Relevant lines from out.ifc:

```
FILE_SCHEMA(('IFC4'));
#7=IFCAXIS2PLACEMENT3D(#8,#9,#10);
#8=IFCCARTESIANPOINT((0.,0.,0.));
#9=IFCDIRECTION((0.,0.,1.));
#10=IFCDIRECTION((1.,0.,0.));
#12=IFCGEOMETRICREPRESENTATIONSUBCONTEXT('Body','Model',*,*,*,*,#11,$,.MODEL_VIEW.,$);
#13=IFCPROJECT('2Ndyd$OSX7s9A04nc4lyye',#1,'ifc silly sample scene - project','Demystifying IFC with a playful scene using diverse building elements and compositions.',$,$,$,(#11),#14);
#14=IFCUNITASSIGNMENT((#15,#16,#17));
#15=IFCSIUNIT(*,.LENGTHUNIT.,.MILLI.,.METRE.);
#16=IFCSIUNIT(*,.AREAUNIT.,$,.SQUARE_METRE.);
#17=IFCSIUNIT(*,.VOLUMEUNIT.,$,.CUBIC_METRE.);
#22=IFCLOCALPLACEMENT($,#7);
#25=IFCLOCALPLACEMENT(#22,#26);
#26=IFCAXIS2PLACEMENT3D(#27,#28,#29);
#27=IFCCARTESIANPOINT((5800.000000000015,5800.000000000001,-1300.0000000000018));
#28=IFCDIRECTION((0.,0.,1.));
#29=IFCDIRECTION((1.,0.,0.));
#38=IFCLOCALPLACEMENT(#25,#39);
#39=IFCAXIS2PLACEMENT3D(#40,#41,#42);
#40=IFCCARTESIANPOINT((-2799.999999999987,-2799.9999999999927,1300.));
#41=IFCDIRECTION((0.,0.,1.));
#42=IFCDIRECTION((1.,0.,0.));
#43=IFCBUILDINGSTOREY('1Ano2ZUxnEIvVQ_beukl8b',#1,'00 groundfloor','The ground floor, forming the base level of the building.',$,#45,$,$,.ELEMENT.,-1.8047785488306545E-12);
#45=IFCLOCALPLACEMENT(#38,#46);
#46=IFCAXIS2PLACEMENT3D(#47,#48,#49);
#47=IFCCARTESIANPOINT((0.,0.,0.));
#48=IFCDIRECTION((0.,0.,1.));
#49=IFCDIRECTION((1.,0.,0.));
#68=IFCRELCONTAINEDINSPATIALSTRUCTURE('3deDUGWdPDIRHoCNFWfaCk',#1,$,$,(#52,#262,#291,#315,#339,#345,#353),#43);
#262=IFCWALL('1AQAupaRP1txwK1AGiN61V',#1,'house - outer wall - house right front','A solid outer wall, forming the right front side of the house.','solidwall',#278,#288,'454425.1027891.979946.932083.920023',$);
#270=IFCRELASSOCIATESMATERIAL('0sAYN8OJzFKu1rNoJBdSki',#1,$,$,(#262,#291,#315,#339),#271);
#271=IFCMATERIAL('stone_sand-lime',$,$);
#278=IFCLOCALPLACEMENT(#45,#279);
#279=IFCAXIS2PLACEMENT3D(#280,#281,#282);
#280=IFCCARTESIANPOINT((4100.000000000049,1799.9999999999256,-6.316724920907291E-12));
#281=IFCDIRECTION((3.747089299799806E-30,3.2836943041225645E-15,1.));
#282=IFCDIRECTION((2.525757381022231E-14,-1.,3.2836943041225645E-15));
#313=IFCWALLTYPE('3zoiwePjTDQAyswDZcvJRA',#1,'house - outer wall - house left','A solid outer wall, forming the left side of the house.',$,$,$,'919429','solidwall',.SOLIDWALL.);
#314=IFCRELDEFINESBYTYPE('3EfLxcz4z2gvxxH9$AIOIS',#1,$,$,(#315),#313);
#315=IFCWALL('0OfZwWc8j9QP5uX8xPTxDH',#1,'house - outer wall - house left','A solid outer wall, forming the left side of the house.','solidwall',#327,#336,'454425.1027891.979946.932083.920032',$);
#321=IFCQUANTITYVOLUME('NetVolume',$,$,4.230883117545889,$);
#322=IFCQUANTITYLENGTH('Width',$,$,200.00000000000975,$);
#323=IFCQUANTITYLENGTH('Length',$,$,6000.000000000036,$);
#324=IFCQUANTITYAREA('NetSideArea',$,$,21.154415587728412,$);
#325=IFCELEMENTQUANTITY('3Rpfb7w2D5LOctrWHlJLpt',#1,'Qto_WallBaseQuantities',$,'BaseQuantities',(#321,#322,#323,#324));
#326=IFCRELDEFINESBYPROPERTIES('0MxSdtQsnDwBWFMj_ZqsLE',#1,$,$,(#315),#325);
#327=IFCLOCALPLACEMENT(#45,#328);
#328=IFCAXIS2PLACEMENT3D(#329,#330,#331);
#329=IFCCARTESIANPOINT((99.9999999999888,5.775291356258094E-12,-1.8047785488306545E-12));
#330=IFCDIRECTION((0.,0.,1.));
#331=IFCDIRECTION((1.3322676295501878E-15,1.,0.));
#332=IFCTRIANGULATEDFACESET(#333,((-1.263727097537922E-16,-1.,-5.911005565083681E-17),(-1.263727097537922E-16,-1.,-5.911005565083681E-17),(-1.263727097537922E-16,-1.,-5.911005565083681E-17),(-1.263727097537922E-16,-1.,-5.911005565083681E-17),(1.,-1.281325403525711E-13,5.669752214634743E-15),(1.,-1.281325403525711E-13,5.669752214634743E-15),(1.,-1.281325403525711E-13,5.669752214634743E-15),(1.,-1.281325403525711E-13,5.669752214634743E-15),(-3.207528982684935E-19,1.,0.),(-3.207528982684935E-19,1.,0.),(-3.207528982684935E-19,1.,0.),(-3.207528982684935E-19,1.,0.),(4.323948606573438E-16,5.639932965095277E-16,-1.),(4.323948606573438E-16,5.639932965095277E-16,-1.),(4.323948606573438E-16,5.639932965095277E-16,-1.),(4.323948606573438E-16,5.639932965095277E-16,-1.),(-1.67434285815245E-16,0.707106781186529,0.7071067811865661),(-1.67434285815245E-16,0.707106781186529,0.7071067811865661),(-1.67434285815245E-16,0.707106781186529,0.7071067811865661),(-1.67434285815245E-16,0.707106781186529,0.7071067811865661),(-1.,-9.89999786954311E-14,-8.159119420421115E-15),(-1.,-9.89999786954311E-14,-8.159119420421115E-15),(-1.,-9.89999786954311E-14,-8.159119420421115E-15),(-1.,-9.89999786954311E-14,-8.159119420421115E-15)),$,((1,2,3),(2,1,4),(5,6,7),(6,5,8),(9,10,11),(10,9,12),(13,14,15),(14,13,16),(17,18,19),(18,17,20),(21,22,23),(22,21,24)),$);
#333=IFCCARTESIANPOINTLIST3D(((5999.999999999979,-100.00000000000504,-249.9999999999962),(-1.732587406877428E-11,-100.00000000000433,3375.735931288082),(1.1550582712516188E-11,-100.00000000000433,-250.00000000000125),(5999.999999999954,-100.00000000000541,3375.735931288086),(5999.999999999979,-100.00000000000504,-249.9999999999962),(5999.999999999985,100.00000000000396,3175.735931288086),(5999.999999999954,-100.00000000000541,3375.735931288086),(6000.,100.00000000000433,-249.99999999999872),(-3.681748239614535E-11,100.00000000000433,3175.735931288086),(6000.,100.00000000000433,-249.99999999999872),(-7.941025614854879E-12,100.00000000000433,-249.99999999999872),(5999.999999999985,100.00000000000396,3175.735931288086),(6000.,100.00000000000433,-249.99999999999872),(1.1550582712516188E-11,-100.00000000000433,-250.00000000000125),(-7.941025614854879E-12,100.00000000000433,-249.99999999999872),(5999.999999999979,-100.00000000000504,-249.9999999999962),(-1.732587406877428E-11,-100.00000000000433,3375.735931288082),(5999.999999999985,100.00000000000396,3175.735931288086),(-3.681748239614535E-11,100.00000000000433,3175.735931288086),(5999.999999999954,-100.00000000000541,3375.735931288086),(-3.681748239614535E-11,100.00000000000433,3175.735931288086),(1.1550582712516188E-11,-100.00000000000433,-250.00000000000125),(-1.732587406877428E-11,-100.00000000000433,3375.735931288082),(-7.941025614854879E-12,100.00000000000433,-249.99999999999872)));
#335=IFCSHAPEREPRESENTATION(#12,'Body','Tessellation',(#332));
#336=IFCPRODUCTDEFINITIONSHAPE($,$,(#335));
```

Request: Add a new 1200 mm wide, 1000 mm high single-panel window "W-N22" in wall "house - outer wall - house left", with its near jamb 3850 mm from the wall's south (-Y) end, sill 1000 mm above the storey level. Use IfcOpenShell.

```python
import numpy as np
import ifcopenshell
import ifcopenshell.api.feature
import ifcopenshell.api.geometry
import ifcopenshell.api.pset
import ifcopenshell.api.root
import ifcopenshell.api.spatial
import ifcopenshell.geom
import ifcopenshell.util.element
import ifcopenshell.util.placement
import ifcopenshell.util.representation
import ifcopenshell.util.shape
import ifcopenshell.util.unit

model = ifcopenshell.open("out.ifc")
unit_scale = ifcopenshell.util.unit.calculate_unit_scale(model)
area_scale = ifcopenshell.util.unit.calculate_unit_scale(model, "AREAUNIT")
volume_scale = ifcopenshell.util.unit.calculate_unit_scale(model, "VOLUMEUNIT")
settings = ifcopenshell.geom.settings()


def volume(element):
    """Net volume in cubic metres, openings subtracted."""
    shape = ifcopenshell.geom.create_shape(settings, element)
    return ifcopenshell.util.shape.get_volume(shape.geometry)


wall = model.by_guid("0OfZwWc8j9QP5uX8xPTxDH")
storey = ifcopenshell.util.element.get_container(wall, ifc_class="IfcBuildingStorey")
context = ifcopenshell.util.representation.get_context(model, "Model", "Body", "MODEL_VIEW")
before = volume(wall)

width, height, from_end, sill = 1.2, 1, 3.85, 1  # metres

# The wall runs along its own X axis, and the end named is its -X end.
wall_shape = ifcopenshell.geom.create_shape(settings, wall)
x, y, z = ifcopenshell.util.shape.get_vertices(wall_shape.geometry).T
start = x.min() + from_end
face, thickness = float(y.min()), float(y.max() - y.min())
wall_matrix = ifcopenshell.util.placement.get_local_placement(wall.ObjectPlacement)
level = ifcopenshell.util.placement.get_local_placement(storey.ObjectPlacement)[2, 3]


def in_wall(x, y):
    """Placement at x, y metres in the wall's axes, at sill height."""
    matrix = wall_matrix.copy()
    matrix[:, 3] = wall_matrix @ np.array([x / unit_scale, y / unit_scale, 0.0, 1.0])
    matrix[2, 3] = level + sill / unit_scale
    return matrix


# Opening: a box that overshoots both wall faces by 50 mm.
opening = ifcopenshell.api.root.create_entity(model, ifc_class="IfcOpeningElement", predefined_type="OPENING")
box = ifcopenshell.api.geometry.add_wall_representation(
    model, context=context, length=width, height=height, thickness=thickness + 0.1
)
ifcopenshell.api.geometry.assign_representation(model, product=opening, representation=box)
ifcopenshell.api.geometry.edit_object_placement(model, product=opening, matrix=in_wall(start, face - 0.05), is_si=False)
ifcopenshell.api.feature.add_feature(model, feature=opening, element=wall)

window = ifcopenshell.api.root.create_entity(model, ifc_class="IfcWindow", name="W-N22", predefined_type="WINDOW")
window.OverallWidth, window.OverallHeight = width / unit_scale, height / unit_scale
window.PartitioningType = "SINGLE_PANEL"
body = ifcopenshell.api.geometry.add_window_representation(
    model,
    context=context,
    overall_width=window.OverallWidth,
    overall_height=window.OverallHeight,
    partition_type="SINGLE_PANEL",
)
ifcopenshell.api.geometry.assign_representation(model, product=window, representation=body)
ifcopenshell.api.spatial.assign_container(model, products=[window], relating_structure=storey)
ifcopenshell.api.feature.add_filling(model, opening=opening, element=window)

# Centre the window in the wall's thickness.
ifcopenshell.api.geometry.edit_object_placement(model, product=window, matrix=in_wall(start, face), is_si=False)
window_shape = ifcopenshell.geom.create_shape(settings, window)
depth = ifcopenshell.util.shape.get_vertices(window_shape.geometry)[:, 1]
offset = face + thickness / 2 - (depth.min() + depth.max()) / 2
ifcopenshell.api.geometry.edit_object_placement(model, product=window, matrix=in_wall(start, offset), is_si=False)

after = volume(wall)

# Update the wall's stored quantities.
qto = model.by_id(ifcopenshell.util.element.get_pset(wall, "Qto_WallBaseQuantities", should_inherit=False)["id"])
ifcopenshell.api.pset.edit_qto(model, qto=qto, properties={
    "NetVolume": after / volume_scale,
    "NetSideArea": after / thickness / area_scale,
})

print(f"wall volume {before:.3f} -> {after:.3f} m3")

model.write("out_rev.ifc")
```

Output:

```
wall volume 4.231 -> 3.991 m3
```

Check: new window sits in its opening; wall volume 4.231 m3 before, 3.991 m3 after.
